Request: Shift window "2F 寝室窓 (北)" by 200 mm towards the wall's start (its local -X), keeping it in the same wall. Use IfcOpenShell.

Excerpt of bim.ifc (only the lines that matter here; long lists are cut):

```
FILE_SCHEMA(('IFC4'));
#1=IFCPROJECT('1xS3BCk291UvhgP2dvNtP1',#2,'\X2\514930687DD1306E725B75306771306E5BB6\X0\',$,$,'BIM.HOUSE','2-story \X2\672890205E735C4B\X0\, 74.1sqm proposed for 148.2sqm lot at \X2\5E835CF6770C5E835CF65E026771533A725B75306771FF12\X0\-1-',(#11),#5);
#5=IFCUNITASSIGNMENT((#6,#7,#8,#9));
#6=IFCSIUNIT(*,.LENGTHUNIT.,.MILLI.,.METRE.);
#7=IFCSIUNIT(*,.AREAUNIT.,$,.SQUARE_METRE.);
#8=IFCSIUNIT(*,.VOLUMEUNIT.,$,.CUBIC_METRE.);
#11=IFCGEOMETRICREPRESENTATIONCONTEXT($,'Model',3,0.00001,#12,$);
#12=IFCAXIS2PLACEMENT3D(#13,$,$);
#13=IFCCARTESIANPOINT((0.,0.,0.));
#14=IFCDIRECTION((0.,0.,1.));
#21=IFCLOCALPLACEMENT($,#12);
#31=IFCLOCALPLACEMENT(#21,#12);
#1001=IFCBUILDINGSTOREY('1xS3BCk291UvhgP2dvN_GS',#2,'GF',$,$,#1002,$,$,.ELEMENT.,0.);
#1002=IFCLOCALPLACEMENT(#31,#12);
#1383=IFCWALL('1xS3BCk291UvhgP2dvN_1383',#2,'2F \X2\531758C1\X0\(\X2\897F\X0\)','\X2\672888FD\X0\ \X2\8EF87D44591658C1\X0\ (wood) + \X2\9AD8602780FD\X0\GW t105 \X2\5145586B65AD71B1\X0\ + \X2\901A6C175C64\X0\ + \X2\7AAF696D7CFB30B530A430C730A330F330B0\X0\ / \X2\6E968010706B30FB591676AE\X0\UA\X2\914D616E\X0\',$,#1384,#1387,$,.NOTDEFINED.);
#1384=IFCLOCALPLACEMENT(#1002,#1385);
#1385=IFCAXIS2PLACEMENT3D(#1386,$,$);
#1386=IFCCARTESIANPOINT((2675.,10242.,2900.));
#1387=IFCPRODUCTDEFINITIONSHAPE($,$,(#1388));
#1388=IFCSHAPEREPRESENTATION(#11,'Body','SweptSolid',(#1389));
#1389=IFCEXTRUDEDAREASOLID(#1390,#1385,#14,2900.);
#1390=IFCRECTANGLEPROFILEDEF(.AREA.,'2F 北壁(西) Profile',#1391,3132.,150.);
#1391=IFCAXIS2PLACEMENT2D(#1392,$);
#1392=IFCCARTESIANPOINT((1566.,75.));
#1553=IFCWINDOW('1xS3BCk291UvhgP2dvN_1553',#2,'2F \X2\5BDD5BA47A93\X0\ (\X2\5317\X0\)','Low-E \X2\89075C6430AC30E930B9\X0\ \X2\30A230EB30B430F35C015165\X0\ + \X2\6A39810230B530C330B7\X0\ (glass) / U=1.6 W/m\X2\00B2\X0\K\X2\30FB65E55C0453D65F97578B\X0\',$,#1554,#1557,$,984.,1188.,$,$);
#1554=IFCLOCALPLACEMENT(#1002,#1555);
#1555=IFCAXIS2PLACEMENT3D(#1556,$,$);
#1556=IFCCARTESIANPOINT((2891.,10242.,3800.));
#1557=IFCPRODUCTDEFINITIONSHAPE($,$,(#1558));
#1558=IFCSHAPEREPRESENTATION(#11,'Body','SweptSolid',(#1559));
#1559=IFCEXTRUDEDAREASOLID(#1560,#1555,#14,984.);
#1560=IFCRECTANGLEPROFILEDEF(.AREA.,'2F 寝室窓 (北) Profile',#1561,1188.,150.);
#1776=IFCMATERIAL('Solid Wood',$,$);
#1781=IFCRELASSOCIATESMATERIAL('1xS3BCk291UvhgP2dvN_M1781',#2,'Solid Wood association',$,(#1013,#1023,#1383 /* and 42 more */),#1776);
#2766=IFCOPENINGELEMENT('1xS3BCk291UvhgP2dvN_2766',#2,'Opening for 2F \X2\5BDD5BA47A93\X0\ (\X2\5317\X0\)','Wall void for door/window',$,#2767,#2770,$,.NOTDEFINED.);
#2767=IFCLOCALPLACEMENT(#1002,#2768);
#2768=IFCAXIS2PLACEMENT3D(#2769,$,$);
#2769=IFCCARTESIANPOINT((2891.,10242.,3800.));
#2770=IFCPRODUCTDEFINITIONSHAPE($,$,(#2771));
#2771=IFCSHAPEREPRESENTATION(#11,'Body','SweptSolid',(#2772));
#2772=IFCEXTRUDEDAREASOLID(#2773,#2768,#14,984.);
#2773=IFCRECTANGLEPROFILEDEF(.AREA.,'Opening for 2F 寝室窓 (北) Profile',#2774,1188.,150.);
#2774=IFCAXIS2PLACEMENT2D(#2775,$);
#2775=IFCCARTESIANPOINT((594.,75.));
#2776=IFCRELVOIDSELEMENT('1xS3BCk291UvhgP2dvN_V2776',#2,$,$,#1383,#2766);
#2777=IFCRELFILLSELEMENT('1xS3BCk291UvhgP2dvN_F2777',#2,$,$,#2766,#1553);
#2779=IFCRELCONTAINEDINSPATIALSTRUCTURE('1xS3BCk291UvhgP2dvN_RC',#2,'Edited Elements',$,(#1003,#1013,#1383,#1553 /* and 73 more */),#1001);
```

```python
import ifcopenshell
import ifcopenshell.api.geometry
import ifcopenshell.util.placement

model = ifcopenshell.open("bim.ifc")

window = model.by_guid("1xS3BCk291UvhgP2dvN_1553")
opening = window.FillsVoids[0].RelatingOpeningElement
wall = opening.VoidsElements[0].RelatingBuildingElement

wall_matrix = ifcopenshell.util.placement.get_local_placement(wall.ObjectPlacement)
shift = wall_matrix[:3, 0] * -200.0
before = ifcopenshell.util.placement.get_local_placement(window.ObjectPlacement)[:3, 3].copy()

# The window is not placed relative to its opening, so move both.
for product in (opening, window):
    matrix = ifcopenshell.util.placement.get_local_placement(product.ObjectPlacement)
    matrix[:3, 3] += shift
    ifcopenshell.api.geometry.edit_object_placement(model, product=product, matrix=matrix, is_si=False)

after = ifcopenshell.util.placement.get_local_placement(window.ObjectPlacement)[:3, 3]
print("window moved by", (after - before).round(3) + 0.0)

model.write("bim_updated.ifc")
```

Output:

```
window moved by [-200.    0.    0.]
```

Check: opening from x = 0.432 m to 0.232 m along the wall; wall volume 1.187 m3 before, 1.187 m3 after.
